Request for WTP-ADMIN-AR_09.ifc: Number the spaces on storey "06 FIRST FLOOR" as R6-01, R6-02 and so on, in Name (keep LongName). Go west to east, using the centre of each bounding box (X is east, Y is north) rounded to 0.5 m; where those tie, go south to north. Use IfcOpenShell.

First a look at what the model holds.

```python
import ifcopenshell
import ifcopenshell.util.element
import ifcopenshell.util.placement

model = ifcopenshell.open("WTP-ADMIN-AR_09.ifc")
print(model.schema)
storey = next(s for s in model.by_type("IfcBuildingStorey") if s.Name == "06 FIRST FLOOR")
spaces = [e for e in ifcopenshell.util.element.get_decomposition(storey) if e.is_a("IfcSpace")]
for e in sorted(spaces, key=lambda e: e.id()):
    origin = ifcopenshell.util.placement.get_local_placement(e.ObjectPlacement)[:3, 3]
    print(e.id(), e.Name, e.LongName, origin.round(2) + 0.0, sep=" | ")
```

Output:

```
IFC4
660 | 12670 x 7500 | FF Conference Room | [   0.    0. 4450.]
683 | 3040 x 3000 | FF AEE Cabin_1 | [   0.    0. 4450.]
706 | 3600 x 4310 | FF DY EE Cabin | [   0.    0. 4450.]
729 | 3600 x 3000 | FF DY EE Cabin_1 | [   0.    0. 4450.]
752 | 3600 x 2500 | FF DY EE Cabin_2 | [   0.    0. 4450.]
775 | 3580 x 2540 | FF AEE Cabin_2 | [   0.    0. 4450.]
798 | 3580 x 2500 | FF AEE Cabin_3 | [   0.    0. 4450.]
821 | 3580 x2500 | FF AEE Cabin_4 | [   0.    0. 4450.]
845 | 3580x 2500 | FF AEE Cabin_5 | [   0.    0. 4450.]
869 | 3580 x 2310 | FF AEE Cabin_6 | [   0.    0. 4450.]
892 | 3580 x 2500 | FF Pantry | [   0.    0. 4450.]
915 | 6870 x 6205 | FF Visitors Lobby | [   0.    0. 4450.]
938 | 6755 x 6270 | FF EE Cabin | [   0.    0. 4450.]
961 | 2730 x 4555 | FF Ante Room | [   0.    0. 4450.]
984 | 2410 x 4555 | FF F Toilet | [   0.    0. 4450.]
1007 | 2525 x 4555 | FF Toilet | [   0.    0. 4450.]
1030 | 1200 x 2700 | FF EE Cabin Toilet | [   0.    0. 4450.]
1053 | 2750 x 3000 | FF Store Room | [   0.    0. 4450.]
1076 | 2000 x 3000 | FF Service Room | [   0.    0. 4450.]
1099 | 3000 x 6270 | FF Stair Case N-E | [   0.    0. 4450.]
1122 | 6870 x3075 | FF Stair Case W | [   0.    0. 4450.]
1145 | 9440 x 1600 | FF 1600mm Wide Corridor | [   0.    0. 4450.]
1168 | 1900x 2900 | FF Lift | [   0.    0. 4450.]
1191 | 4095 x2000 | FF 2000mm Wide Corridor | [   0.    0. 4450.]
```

```python
import ifcopenshell
import ifcopenshell.geom
import ifcopenshell.util.element
import ifcopenshell.util.shape

model = ifcopenshell.open("WTP-ADMIN-AR_09.ifc")
settings = ifcopenshell.geom.settings()
settings.set("use-world-coords", True)


def centre(element):
    shape = ifcopenshell.geom.create_shape(settings, element)
    return ifcopenshell.util.shape.get_bbox_centroid(shape.geometry)


storey = next(s for s in model.by_type("IfcBuildingStorey") if s.Name == "06 FIRST FLOOR")
spaces = [e for e in ifcopenshell.util.element.get_decomposition(storey) if e.is_a("IfcSpace")]

# Insertion points can sit at a corner or the storey origin, so sort by the geometry (in metres).
centres = {e: centre(e) for e in spaces}
spaces.sort(key=lambda e: (round(centres[e][0] / 0.5), centres[e][1]))

for i, e in enumerate(spaces, start=1):
    number = f"R6-{i:02d}"
    e.Name = number
    print(e.id(), number)

model.write("WTP-ADMIN-AR_09_v2.ifc")
```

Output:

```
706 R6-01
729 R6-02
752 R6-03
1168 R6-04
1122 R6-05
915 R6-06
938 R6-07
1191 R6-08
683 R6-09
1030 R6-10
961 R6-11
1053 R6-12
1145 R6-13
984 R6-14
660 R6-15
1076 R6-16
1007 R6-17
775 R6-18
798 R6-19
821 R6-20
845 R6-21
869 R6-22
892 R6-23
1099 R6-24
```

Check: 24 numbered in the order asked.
